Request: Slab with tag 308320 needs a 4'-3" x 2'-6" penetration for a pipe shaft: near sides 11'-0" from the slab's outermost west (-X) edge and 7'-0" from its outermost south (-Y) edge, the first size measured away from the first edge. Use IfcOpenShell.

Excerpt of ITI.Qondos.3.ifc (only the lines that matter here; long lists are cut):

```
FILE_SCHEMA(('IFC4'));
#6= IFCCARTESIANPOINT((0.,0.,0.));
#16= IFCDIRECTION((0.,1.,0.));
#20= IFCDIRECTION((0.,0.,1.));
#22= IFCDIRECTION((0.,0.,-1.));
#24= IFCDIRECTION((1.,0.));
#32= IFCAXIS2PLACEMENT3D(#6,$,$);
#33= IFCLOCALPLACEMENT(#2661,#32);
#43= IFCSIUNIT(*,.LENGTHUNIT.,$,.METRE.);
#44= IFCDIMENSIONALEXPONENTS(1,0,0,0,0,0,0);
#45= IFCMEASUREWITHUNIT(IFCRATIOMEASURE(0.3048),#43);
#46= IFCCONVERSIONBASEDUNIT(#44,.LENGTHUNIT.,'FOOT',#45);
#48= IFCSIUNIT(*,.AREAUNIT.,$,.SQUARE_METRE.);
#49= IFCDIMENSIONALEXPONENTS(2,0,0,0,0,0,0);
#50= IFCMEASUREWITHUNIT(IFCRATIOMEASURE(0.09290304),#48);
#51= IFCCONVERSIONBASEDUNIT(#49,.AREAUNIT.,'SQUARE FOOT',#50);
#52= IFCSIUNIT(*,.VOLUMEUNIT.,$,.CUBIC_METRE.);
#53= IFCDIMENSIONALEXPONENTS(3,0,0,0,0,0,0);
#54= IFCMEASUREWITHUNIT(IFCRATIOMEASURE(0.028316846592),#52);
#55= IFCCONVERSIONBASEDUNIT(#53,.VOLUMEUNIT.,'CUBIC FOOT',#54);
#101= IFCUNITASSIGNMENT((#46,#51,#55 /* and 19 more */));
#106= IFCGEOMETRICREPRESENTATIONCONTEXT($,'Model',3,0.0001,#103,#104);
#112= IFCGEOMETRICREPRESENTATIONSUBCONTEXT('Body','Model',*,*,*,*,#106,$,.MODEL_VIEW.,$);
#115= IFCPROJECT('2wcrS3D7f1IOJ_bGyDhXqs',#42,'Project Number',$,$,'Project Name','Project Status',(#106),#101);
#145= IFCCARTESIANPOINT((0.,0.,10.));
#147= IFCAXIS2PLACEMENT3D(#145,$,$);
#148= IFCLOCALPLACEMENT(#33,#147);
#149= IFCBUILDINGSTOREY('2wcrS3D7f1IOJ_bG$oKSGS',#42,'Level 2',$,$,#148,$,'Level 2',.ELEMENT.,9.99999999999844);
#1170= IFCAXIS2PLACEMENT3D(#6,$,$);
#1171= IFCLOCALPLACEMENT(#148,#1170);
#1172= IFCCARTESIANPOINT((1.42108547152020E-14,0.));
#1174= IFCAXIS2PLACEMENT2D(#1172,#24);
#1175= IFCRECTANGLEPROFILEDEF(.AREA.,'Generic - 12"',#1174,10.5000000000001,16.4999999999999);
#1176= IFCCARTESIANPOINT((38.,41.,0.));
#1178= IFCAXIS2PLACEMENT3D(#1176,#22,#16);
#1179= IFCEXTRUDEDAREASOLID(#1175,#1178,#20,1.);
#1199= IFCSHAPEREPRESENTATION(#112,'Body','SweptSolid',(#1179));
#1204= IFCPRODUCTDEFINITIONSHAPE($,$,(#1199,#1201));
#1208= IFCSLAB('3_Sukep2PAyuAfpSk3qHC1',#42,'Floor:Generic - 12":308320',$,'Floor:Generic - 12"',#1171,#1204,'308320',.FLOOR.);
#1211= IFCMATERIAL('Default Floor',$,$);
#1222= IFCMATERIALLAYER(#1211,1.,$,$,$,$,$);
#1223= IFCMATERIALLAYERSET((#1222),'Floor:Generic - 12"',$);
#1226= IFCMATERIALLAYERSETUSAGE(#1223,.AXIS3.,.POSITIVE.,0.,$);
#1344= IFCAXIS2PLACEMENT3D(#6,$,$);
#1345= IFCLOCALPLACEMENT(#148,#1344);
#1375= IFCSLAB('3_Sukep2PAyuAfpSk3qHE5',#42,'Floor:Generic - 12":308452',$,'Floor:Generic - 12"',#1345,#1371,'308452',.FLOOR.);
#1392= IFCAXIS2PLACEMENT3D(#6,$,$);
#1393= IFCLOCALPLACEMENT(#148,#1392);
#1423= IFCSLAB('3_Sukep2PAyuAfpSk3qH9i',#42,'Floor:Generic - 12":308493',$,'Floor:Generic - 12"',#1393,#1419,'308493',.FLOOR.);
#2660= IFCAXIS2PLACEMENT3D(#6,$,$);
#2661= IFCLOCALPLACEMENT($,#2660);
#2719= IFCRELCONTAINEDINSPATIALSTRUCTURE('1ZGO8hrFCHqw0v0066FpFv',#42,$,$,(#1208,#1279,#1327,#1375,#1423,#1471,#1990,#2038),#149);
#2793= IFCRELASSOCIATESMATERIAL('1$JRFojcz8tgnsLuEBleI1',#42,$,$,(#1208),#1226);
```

```python
import numpy as np
import ifcopenshell
import ifcopenshell.api.feature
import ifcopenshell.api.geometry
import ifcopenshell.api.root
import ifcopenshell.geom
import ifcopenshell.util.placement
import ifcopenshell.util.representation
import ifcopenshell.util.shape
import ifcopenshell.util.unit

model = ifcopenshell.open("ITI.Qondos.3.ifc")
unit_scale = ifcopenshell.util.unit.calculate_unit_scale(model)
settings = ifcopenshell.geom.settings()


def volume(element):
    """Net volume in cubic metres, openings subtracted."""
    shape = ifcopenshell.geom.create_shape(settings, element)
    return ifcopenshell.util.shape.get_volume(shape.geometry)


slab = model.by_guid("3_Sukep2PAyuAfpSk3qHC1")
before = volume(slab)

# Extent in the slab's own axes, in metres. The edges named are its -X and -Y sides.
slab_shape = ifcopenshell.geom.create_shape(settings, slab)
vertices = ifcopenshell.util.shape.get_vertices(slab_shape.geometry)
x_min, y_min, bottom = vertices.min(axis=0)
top = vertices[:, 2].max()

opening = ifcopenshell.api.root.create_entity(model, ifc_class="IfcOpeningElement", name="Pipe shaft opening", predefined_type="OPENING")
context = ifcopenshell.util.representation.get_context(model, "Model", "Body", "MODEL_VIEW")
width, depth = 1.2954, 0.762
outline = [(0.0, 0.0), (width, 0.0), (width, depth), (0.0, depth), (0.0, 0.0)]
# Overshoot both faces by 50 mm so the cut is clean.
shape = ifcopenshell.api.geometry.add_slab_representation(
    model, context=context, depth=top - bottom + 0.1, polyline=outline
)
ifcopenshell.api.geometry.assign_representation(model, product=opening, representation=shape)

matrix = ifcopenshell.util.placement.get_local_placement(slab.ObjectPlacement)
matrix[:, 3] = matrix @ np.append(np.array([x_min + 3.3528, y_min + 2.1336, bottom - 0.05]) / unit_scale, 1.0)
ifcopenshell.api.geometry.edit_object_placement(model, product=opening, matrix=matrix, is_si=False)
ifcopenshell.api.feature.add_feature(model, feature=opening, element=slab)

after = volume(slab)

print(f"slab volume {before:.3f} -> {after:.3f} m3")

model.write("ITI.Qondos.3_edited.ifc")
```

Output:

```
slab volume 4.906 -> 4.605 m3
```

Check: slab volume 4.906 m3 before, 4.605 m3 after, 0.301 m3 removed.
